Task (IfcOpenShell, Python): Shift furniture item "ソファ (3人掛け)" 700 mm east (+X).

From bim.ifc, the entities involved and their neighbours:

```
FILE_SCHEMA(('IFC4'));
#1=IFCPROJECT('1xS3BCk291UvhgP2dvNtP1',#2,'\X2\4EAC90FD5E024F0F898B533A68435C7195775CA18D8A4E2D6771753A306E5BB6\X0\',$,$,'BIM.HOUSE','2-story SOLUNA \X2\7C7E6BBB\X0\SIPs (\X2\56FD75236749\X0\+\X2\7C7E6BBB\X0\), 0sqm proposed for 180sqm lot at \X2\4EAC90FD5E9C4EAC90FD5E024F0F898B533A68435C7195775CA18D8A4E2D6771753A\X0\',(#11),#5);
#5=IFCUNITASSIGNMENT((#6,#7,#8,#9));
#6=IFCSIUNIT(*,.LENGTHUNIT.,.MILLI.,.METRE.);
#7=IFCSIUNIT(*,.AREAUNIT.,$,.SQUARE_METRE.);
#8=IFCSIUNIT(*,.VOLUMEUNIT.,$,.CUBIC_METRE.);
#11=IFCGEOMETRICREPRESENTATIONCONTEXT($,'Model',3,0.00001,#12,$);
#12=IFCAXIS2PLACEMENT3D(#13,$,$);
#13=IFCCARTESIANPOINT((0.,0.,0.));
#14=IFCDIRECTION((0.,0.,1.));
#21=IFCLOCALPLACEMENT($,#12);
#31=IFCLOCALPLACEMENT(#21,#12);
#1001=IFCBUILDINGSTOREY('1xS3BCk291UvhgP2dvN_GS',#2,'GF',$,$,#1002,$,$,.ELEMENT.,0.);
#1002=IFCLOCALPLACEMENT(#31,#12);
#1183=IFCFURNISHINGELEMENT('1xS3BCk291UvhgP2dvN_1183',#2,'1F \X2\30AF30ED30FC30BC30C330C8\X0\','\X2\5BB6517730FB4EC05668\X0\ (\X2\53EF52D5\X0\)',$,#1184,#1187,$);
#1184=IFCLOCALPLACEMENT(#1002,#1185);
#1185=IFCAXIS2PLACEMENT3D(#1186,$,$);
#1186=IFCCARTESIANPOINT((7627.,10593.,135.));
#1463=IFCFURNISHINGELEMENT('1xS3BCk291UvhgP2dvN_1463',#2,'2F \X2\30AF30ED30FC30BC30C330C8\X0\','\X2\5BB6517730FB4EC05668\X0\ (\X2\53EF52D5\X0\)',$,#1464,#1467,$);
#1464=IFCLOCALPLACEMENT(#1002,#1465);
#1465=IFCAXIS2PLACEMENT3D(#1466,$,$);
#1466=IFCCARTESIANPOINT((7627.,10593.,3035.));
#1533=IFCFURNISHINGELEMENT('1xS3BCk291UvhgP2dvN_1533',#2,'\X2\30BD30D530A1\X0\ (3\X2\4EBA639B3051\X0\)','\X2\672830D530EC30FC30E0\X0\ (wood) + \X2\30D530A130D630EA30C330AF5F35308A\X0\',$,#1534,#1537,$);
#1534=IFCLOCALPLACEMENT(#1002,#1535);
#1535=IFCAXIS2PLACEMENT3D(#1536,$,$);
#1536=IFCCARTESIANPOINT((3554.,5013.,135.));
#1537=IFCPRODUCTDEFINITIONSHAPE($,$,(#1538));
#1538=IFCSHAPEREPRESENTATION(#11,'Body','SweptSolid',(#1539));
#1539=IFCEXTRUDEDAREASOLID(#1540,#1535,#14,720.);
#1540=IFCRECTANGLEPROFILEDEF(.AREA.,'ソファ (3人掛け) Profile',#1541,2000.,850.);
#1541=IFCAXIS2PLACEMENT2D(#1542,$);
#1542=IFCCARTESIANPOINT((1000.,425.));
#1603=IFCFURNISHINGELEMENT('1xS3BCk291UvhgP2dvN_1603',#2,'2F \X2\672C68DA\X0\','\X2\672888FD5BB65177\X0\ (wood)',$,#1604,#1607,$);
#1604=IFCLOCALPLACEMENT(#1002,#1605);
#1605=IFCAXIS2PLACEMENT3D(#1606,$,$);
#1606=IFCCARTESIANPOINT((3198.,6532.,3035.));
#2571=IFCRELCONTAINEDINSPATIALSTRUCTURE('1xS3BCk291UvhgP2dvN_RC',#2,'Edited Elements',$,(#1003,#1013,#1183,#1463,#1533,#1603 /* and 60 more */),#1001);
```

```python
import ifcopenshell
import ifcopenshell.api.geometry
import ifcopenshell.util.placement
import ifcopenshell.util.unit

model = ifcopenshell.open("bim.ifc")
unit_scale = ifcopenshell.util.unit.calculate_unit_scale(model)

item = model.by_guid("1xS3BCk291UvhgP2dvN_1533")
matrix = ifcopenshell.util.placement.get_local_placement(item.ObjectPlacement)
matrix[0, 3] += 0.7 / unit_scale
ifcopenshell.api.geometry.edit_object_placement(model, product=item, matrix=matrix, is_si=False)

print(ifcopenshell.util.placement.get_local_placement(item.ObjectPlacement).round(3) + 0.0)

model.write("bim_updated.ifc")
```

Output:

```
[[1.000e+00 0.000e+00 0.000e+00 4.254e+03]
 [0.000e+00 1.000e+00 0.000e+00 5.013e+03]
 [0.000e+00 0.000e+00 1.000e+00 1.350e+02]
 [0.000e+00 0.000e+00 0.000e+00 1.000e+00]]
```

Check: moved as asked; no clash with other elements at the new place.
